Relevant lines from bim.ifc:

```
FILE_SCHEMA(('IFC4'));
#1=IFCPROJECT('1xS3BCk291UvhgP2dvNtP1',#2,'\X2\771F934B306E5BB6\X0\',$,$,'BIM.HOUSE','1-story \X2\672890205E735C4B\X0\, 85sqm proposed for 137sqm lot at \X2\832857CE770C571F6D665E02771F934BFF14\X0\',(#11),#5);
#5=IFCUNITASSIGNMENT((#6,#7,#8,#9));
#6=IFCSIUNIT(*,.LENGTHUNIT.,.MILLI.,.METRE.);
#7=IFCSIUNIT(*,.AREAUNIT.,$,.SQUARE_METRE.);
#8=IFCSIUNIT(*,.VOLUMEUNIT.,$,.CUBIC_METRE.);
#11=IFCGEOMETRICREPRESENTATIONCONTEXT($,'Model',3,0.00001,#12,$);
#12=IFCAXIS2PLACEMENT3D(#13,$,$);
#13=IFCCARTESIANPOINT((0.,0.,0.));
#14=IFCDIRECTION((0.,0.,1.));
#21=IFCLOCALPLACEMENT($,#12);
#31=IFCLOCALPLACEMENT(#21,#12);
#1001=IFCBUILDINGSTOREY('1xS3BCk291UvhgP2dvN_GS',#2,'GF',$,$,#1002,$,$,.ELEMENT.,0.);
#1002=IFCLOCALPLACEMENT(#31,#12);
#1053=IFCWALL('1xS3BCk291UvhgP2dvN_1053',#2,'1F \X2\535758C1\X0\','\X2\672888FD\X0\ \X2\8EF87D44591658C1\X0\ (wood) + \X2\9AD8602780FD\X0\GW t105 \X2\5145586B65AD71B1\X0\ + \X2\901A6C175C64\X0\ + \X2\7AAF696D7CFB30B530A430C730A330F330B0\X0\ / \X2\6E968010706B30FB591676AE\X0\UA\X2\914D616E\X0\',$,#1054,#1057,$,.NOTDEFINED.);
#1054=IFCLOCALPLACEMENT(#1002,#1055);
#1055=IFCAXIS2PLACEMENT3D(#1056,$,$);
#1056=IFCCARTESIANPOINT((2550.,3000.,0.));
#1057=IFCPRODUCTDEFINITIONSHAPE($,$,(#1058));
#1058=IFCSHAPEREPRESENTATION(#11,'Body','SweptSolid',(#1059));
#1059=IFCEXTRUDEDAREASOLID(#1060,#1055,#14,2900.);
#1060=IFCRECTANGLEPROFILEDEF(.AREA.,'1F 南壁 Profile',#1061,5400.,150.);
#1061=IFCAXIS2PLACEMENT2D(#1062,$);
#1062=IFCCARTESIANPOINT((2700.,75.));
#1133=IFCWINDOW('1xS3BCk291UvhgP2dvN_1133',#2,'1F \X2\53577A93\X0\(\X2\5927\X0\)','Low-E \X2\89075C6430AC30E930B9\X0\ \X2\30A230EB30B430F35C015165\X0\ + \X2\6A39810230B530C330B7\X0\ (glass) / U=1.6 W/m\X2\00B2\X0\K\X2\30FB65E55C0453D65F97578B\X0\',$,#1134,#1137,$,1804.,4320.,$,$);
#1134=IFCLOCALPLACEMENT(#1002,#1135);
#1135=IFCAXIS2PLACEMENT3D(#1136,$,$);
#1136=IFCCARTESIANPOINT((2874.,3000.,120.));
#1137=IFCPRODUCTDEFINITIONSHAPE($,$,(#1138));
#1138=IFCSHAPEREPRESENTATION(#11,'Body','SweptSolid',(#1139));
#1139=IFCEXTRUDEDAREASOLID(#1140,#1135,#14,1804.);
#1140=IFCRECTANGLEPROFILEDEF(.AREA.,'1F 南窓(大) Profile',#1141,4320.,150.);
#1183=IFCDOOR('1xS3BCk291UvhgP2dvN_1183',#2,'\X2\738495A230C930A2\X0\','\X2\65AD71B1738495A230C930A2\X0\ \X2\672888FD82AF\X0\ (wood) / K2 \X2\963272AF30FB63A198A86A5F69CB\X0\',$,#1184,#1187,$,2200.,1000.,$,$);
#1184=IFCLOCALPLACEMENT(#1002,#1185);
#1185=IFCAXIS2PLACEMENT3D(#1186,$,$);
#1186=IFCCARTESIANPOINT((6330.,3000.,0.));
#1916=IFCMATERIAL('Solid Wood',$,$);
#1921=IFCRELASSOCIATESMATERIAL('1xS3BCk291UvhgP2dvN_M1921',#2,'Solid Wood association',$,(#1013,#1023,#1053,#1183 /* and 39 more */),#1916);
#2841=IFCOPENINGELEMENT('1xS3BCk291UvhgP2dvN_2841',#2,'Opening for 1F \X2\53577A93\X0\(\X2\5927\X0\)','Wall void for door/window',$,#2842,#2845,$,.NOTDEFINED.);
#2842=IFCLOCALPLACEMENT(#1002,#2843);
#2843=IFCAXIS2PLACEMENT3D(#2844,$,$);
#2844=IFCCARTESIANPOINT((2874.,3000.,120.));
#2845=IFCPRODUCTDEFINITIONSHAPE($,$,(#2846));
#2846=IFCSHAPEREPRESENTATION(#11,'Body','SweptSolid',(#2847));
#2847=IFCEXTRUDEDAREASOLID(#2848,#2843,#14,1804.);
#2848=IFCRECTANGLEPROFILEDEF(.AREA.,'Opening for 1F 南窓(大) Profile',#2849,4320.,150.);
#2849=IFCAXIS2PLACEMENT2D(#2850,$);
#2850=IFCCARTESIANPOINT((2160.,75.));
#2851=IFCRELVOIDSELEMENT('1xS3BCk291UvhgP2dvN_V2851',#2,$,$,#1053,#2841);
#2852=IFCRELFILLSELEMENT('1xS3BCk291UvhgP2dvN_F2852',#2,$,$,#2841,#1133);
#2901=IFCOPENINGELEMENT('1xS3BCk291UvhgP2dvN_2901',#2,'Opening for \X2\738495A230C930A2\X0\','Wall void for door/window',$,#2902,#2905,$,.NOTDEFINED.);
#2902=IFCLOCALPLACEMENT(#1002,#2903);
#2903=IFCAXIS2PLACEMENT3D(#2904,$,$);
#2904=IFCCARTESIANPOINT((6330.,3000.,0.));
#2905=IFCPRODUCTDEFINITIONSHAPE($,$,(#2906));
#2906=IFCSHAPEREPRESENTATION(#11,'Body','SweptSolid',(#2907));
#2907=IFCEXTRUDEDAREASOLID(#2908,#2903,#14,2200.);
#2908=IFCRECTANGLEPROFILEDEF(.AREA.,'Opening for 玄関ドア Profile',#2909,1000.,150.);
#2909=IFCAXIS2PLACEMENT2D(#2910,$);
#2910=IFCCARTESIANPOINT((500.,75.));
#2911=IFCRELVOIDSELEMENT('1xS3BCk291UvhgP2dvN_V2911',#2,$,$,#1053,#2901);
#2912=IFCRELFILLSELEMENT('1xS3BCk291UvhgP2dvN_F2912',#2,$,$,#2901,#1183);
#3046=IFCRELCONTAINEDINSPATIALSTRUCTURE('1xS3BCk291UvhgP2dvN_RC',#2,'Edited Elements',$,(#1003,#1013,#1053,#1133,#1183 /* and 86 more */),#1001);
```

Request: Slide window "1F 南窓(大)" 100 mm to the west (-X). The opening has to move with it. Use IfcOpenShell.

```python
import ifcopenshell
import ifcopenshell.api.geometry
import ifcopenshell.util.placement
import ifcopenshell.util.unit

model = ifcopenshell.open("bim.ifc")
unit_scale = ifcopenshell.util.unit.calculate_unit_scale(model)

window = model.by_guid("1xS3BCk291UvhgP2dvN_1133")
opening = window.FillsVoids[0].RelatingOpeningElement
wall = opening.VoidsElements[0].RelatingBuildingElement

wall_matrix = ifcopenshell.util.placement.get_local_placement(wall.ObjectPlacement)
shift = wall_matrix[:3, 0] * -0.1 / unit_scale
before = ifcopenshell.util.placement.get_local_placement(window.ObjectPlacement)[:3, 3].copy()

# The window is not placed relative to its opening, so move both.
for product in (opening, window):
    matrix = ifcopenshell.util.placement.get_local_placement(product.ObjectPlacement)
    matrix[:3, 3] += shift
    ifcopenshell.api.geometry.edit_object_placement(model, product=product, matrix=matrix, is_si=False)

after = ifcopenshell.util.placement.get_local_placement(window.ObjectPlacement)[:3, 3]
print("window moved by", (after - before).round(3) + 0.0)

model.write("bim-out.ifc")
```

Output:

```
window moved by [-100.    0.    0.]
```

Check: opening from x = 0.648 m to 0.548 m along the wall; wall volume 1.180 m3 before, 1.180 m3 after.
